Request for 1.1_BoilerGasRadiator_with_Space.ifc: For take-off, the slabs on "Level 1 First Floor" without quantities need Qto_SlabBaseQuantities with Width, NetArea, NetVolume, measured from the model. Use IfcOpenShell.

First a look at what the model holds.

```python
import ifcopenshell
import ifcopenshell.util.element
import ifcopenshell.util.unit

model = ifcopenshell.open("1.1_BoilerGasRadiator_with_Space.ifc")
print(model.schema)
for unit_type in ("LENGTHUNIT", "AREAUNIT", "VOLUMEUNIT"):
    print(unit_type, ifcopenshell.util.unit.calculate_unit_scale(model, unit_type))
storey = next(s for s in model.by_type("IfcBuildingStorey") if s.Name == "Level 1 First Floor")
slabs = [e for e in ifcopenshell.util.element.get_decomposition(storey) if e.is_a("IfcSlab")]
for e in sorted(slabs, key=lambda e: e.id()):
    print(e.id(), e.is_a(), e.Name, list(ifcopenshell.util.element.get_psets(e, qtos_only=True)), sep=" | ")
```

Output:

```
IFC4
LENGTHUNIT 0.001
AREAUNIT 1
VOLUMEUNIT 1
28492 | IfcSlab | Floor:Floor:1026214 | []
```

```python
import ifcopenshell
import ifcopenshell.api.pset
import ifcopenshell.geom
import ifcopenshell.util.element
import ifcopenshell.util.shape
import ifcopenshell.util.unit

model = ifcopenshell.open("1.1_BoilerGasRadiator_with_Space.ifc")
unit_scale = ifcopenshell.util.unit.calculate_unit_scale(model)
area_scale = ifcopenshell.util.unit.calculate_unit_scale(model, "AREAUNIT")
volume_scale = ifcopenshell.util.unit.calculate_unit_scale(model, "VOLUMEUNIT")
settings = ifcopenshell.geom.settings()

storey = next(s for s in model.by_type("IfcBuildingStorey") if s.Name == "Level 1 First Floor")
slabs = [e for e in ifcopenshell.util.element.get_decomposition(storey) if e.is_a("IfcSlab")]

for e in sorted(slabs, key=lambda e: e.id()):
    if ifcopenshell.util.element.get_psets(e, qtos_only=True, should_inherit=False):
        continue
    # Geometry comes back in metres, in the element's own axes.
    shape = ifcopenshell.geom.create_shape(settings, e)
    values = {
        "Width": ifcopenshell.util.shape.get_z(shape.geometry) / unit_scale,
        "NetArea": ifcopenshell.util.shape.get_footprint_area(shape.geometry) / area_scale,
        "NetVolume": ifcopenshell.util.shape.get_volume(shape.geometry) / volume_scale,
    }
    qto = ifcopenshell.api.pset.add_qto(model, product=e, name="Qto_SlabBaseQuantities")
    ifcopenshell.api.pset.edit_qto(model, qto=qto, properties=values)
    print(e.id(), {k: round(v, 3) for k, v in values.items()})

model.write("1.1_BoilerGasRadiator_with_Space_v2.ifc")
```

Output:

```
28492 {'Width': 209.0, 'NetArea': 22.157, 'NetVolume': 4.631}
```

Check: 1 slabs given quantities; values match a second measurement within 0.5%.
